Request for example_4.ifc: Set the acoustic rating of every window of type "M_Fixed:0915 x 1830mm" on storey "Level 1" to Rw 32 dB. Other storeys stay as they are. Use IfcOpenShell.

First a look at what the model holds.

```python
import ifcopenshell
import ifcopenshell.util.element

model = ifcopenshell.open("example_4.ifc")
print(model.schema)
storey = next(s for s in model.by_type("IfcBuildingStorey") if s.Name == "Level 1")
windows = [e for e in ifcopenshell.util.element.get_decomposition(storey) if e.is_a("IfcWindow")]
seen = {}
for e in windows:
    element_type = ifcopenshell.util.element.get_type(e)
    key = (element_type.Name if element_type != e and element_type else None, ifcopenshell.util.element.get_pset(e, "Pset_WindowCommon", "AcousticRating"))
    seen[key] = seen.get(key, 0) + 1
for (name, value), count in sorted(seen.items(), key=str):
    print(count, "x", name, "|", value)
```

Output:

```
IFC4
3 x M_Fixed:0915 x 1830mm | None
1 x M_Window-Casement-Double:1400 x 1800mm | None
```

```python
import ifcopenshell
import ifcopenshell.api.pset
import ifcopenshell.util.element

model = ifcopenshell.open("example_4.ifc")

storey = next(s for s in model.by_type("IfcBuildingStorey") if s.Name == "Level 1")
windows = [e for e in ifcopenshell.util.element.get_decomposition(storey) if e.is_a("IfcWindow")]

count = 0
for e in windows:
    element_type = ifcopenshell.util.element.get_type(e)
    if element_type in (None, e) or element_type.Name != "M_Fixed:0915 x 1830mm":
        continue
    # add_pset returns the element's existing set when there is one.
    pset = ifcopenshell.api.pset.add_pset(model, product=e, name="Pset_WindowCommon")
    ifcopenshell.api.pset.edit_pset(model, pset=pset, properties={"AcousticRating": "Rw 32 dB"})
    count += 1

print(count, "windows updated")

model.write("example_4_rev.ifc")
```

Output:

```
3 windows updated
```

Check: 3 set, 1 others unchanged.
